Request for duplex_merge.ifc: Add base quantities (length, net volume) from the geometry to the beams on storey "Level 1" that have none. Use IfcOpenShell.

First a look at what the model holds.

```python
import ifcopenshell
import ifcopenshell.util.element
import ifcopenshell.util.unit

model = ifcopenshell.open("duplex_merge.ifc")
print(model.schema)
for unit_type in ("LENGTHUNIT", "AREAUNIT", "VOLUMEUNIT"):
    print(unit_type, ifcopenshell.util.unit.calculate_unit_scale(model, unit_type))
storey = next(s for s in model.by_type("IfcBuildingStorey") if s.Name == "Level 1")
beams = [e for e in ifcopenshell.util.element.get_decomposition(storey) if e.is_a("IfcBeam")]
for e in sorted(beams, key=lambda e: e.id()):
    print(e.id(), e.is_a(), e.Name, list(ifcopenshell.util.element.get_psets(e, qtos_only=True)), sep=" | ")
```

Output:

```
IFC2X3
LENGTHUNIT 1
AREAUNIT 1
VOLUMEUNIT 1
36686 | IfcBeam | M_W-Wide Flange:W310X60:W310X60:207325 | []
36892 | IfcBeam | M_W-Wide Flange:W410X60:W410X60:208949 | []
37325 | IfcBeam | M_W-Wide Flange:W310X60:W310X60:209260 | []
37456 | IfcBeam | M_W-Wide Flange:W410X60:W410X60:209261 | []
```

```python
import ifcopenshell
import ifcopenshell.api.pset
import ifcopenshell.geom
import ifcopenshell.util.element
import ifcopenshell.util.shape
import ifcopenshell.util.unit

model = ifcopenshell.open("duplex_merge.ifc")
unit_scale = ifcopenshell.util.unit.calculate_unit_scale(model)
volume_scale = ifcopenshell.util.unit.calculate_unit_scale(model, "VOLUMEUNIT")
settings = ifcopenshell.geom.settings()

storey = next(s for s in model.by_type("IfcBuildingStorey") if s.Name == "Level 1")
beams = [e for e in ifcopenshell.util.element.get_decomposition(storey) if e.is_a("IfcBeam")]

for e in sorted(beams, key=lambda e: e.id()):
    if ifcopenshell.util.element.get_psets(e, qtos_only=True, should_inherit=False):
        continue
    # Geometry comes back in metres, in the element's own axes.
    shape = ifcopenshell.geom.create_shape(settings, e)
    values = {
        "Length": ifcopenshell.util.shape.get_max_xyz(shape.geometry) / unit_scale,
        "NetVolume": ifcopenshell.util.shape.get_volume(shape.geometry) / volume_scale,
    }
    qto = ifcopenshell.api.pset.add_qto(model, product=e, name="BaseQuantities")
    ifcopenshell.api.pset.edit_qto(model, qto=qto, properties=values)
    print(e.id(), {k: round(v, 3) for k, v in values.items()})

model.write("duplex_merge_updated.ifc")
```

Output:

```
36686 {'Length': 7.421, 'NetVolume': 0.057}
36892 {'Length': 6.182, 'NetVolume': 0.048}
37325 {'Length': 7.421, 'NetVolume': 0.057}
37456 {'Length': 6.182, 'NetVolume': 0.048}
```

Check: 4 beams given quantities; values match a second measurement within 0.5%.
